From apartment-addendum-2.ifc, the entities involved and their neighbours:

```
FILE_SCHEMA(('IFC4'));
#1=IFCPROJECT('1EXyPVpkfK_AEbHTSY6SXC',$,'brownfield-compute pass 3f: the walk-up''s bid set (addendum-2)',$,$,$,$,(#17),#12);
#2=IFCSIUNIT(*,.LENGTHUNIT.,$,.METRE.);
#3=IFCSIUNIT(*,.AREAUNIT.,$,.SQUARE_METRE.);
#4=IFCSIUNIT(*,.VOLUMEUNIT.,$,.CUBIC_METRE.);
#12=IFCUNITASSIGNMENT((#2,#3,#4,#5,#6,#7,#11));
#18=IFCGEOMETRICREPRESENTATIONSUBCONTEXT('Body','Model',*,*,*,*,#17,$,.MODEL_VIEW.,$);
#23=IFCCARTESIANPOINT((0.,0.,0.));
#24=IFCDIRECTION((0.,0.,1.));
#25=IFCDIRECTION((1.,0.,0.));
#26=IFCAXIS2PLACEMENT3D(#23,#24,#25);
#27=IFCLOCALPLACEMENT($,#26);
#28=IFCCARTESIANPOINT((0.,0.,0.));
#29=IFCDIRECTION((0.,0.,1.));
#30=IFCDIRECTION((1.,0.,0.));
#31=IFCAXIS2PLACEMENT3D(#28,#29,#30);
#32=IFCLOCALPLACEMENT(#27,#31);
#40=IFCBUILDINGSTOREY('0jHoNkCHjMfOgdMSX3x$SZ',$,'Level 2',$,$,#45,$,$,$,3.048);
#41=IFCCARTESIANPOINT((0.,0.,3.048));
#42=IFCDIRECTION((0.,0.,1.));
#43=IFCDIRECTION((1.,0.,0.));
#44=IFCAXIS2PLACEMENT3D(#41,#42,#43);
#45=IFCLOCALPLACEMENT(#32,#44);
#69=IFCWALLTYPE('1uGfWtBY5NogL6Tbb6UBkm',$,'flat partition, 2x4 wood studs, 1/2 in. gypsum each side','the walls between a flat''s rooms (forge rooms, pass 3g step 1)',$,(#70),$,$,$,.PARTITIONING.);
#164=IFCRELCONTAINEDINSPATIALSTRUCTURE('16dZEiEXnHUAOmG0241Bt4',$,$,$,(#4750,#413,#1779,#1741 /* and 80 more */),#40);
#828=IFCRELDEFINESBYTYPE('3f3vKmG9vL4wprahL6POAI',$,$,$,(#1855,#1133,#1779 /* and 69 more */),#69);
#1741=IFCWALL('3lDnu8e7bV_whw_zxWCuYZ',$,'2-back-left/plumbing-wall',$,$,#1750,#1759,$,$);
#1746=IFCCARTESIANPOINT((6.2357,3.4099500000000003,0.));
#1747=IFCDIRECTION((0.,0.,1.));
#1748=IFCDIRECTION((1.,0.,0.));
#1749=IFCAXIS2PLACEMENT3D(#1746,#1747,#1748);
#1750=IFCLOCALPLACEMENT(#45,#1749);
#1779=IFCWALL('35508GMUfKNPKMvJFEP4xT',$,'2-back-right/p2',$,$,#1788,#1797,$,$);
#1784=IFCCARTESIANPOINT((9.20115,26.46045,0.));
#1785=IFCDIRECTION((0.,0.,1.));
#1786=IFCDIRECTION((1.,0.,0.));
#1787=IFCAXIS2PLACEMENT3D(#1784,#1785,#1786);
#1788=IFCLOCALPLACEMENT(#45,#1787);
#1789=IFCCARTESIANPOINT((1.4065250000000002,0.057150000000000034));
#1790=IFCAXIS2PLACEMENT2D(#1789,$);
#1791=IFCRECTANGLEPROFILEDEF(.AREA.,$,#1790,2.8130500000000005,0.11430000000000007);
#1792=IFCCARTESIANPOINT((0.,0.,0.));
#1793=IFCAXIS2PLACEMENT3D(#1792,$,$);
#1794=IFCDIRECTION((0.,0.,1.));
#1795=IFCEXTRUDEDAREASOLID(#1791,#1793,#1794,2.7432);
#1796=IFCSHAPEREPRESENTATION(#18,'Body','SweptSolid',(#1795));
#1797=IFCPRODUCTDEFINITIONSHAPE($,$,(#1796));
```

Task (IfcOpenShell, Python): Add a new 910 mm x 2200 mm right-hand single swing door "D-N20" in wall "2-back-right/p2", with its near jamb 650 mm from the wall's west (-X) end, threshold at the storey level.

```python
import numpy as np
import ifcopenshell
import ifcopenshell.api.feature
import ifcopenshell.api.geometry
import ifcopenshell.api.root
import ifcopenshell.api.spatial
import ifcopenshell.geom
import ifcopenshell.util.element
import ifcopenshell.util.placement
import ifcopenshell.util.representation
import ifcopenshell.util.shape
import ifcopenshell.util.unit

model = ifcopenshell.open("apartment-addendum-2.ifc")
unit_scale = ifcopenshell.util.unit.calculate_unit_scale(model)
settings = ifcopenshell.geom.settings()


def volume(element):
    """Net volume in cubic metres, openings subtracted."""
    shape = ifcopenshell.geom.create_shape(settings, element)
    return ifcopenshell.util.shape.get_volume(shape.geometry)


wall = model.by_guid("35508GMUfKNPKMvJFEP4xT")
storey = ifcopenshell.util.element.get_container(wall, ifc_class="IfcBuildingStorey")
context = ifcopenshell.util.representation.get_context(model, "Model", "Body", "MODEL_VIEW")
before = volume(wall)

width, height, from_end, sill = 0.91, 2.2, 0.65, 0.0  # metres

# The wall runs along its own X axis, and the end named is its -X end.
wall_shape = ifcopenshell.geom.create_shape(settings, wall)
x, y, z = ifcopenshell.util.shape.get_vertices(wall_shape.geometry).T
start = x.min() + from_end
face, thickness = float(y.min()), float(y.max() - y.min())
wall_matrix = ifcopenshell.util.placement.get_local_placement(wall.ObjectPlacement)
level = ifcopenshell.util.placement.get_local_placement(storey.ObjectPlacement)[2, 3]


def in_wall(x, y):
    """Placement at x, y metres in the wall's axes, at sill height."""
    matrix = wall_matrix.copy()
    matrix[:, 3] = wall_matrix @ np.array([x / unit_scale, y / unit_scale, 0.0, 1.0])
    matrix[2, 3] = level + sill / unit_scale
    return matrix


# Opening: a box that overshoots both wall faces by 50 mm.
opening = ifcopenshell.api.root.create_entity(model, ifc_class="IfcOpeningElement", predefined_type="OPENING")
box = ifcopenshell.api.geometry.add_wall_representation(
    model, context=context, length=width, height=height, thickness=thickness + 0.1
)
ifcopenshell.api.geometry.assign_representation(model, product=opening, representation=box)
ifcopenshell.api.geometry.edit_object_placement(model, product=opening, matrix=in_wall(start, face - 0.05), is_si=False)
ifcopenshell.api.feature.add_feature(model, feature=opening, element=wall)

door = ifcopenshell.api.root.create_entity(model, ifc_class="IfcDoor", name="D-N20", predefined_type="DOOR")
door.OverallWidth, door.OverallHeight = width / unit_scale, height / unit_scale
door.OperationType = "SINGLE_SWING_RIGHT"
body = ifcopenshell.api.geometry.add_door_representation(
    model,
    context=context,
    overall_width=door.OverallWidth,
    overall_height=door.OverallHeight,
    operation_type="SINGLE_SWING_RIGHT",
    lining_properties={"LiningDepth": thickness / unit_scale, "ThresholdDepth": thickness / unit_scale},
)
ifcopenshell.api.geometry.assign_representation(model, product=door, representation=body)
ifcopenshell.api.spatial.assign_container(model, products=[door], relating_structure=storey)
ifcopenshell.api.feature.add_filling(model, opening=opening, element=door)

# The lining spans the wall, so the door starts at the wall face.
ifcopenshell.api.geometry.edit_object_placement(model, product=door, matrix=in_wall(start, face), is_si=False)

after = volume(wall)

print(f"wall volume {before:.3f} -> {after:.3f} m3")

model.write("apartment-addendum-2_rev.ifc")
```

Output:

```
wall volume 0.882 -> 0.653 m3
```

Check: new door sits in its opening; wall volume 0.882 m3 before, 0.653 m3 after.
